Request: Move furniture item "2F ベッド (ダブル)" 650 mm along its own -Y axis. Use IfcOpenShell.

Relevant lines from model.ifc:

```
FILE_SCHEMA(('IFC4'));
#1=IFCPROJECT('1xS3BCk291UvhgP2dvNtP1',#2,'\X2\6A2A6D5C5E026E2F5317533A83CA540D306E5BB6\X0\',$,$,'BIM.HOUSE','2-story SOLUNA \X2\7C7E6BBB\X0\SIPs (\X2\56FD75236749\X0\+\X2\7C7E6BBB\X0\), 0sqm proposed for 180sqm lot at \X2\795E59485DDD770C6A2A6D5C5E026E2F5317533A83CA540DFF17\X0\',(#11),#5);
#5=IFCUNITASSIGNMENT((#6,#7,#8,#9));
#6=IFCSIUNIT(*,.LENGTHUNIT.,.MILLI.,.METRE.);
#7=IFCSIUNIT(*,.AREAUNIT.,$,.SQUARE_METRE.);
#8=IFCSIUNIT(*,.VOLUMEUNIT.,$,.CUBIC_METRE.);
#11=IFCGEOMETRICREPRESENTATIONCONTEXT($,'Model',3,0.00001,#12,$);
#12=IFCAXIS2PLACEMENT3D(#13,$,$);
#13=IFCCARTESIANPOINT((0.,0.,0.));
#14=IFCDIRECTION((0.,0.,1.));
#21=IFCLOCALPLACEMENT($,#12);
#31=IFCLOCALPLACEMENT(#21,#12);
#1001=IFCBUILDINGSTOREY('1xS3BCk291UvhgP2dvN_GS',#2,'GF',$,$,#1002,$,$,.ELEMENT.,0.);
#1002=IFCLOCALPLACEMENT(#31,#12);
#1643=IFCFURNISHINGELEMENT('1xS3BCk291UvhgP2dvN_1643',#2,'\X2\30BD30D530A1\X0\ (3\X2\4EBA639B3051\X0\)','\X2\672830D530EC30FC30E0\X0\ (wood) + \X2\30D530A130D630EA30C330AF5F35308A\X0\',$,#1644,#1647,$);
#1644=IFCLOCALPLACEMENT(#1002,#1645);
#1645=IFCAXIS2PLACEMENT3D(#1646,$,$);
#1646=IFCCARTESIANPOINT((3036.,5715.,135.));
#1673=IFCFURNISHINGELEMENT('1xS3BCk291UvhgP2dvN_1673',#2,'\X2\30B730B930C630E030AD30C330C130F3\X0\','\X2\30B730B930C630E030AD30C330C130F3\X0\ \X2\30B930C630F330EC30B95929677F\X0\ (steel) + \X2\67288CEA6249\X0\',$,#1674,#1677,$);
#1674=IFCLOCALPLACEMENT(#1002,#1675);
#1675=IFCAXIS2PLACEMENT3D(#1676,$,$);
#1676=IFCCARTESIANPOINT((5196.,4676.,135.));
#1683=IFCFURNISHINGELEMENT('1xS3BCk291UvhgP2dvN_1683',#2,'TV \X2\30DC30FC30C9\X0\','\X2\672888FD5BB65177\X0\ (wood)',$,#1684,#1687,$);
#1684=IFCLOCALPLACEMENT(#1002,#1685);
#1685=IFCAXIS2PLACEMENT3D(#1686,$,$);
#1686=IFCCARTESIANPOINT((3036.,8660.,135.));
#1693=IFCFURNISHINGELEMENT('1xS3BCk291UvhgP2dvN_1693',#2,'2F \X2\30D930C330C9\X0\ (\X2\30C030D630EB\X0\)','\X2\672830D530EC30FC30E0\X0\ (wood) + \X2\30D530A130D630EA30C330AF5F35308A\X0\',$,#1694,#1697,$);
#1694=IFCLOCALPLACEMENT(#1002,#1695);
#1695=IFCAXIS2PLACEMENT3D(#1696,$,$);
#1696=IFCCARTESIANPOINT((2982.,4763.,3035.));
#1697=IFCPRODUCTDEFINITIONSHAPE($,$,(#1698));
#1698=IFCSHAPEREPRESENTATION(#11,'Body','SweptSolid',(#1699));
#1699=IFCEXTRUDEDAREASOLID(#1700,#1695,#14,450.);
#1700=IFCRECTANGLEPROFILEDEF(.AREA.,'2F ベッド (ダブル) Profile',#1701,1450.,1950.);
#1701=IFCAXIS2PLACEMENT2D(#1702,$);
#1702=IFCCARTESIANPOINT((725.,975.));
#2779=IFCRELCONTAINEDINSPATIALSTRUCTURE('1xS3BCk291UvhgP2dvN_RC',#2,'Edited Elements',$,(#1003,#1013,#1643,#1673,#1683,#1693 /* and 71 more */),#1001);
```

```python
import ifcopenshell
import ifcopenshell.api.geometry
import ifcopenshell.util.placement
import ifcopenshell.util.unit

model = ifcopenshell.open("model.ifc")
unit_scale = ifcopenshell.util.unit.calculate_unit_scale(model)

item = model.by_guid("1xS3BCk291UvhgP2dvN_1693")
matrix = ifcopenshell.util.placement.get_local_placement(item.ObjectPlacement)
matrix[:3, 3] -= matrix[:3, 1] * 0.65 / unit_scale
ifcopenshell.api.geometry.edit_object_placement(model, product=item, matrix=matrix, is_si=False)

print(ifcopenshell.util.placement.get_local_placement(item.ObjectPlacement).round(3) + 0.0)

model.write("model_edited.ifc")
```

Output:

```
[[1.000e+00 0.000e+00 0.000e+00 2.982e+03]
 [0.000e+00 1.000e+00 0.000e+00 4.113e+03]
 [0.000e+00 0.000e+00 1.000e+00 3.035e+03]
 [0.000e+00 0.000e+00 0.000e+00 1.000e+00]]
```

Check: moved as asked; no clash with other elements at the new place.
